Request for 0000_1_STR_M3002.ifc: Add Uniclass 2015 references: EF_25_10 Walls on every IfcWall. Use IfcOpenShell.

First a look at what the model holds.

```python
import ifcopenshell

model = ifcopenshell.open("0000_1_STR_M3002.ifc")
print(model.schema)
print("classifications:", [c.Name for c in model.by_type("IfcClassification")])
for ifc_class in ("IfcDoor", "IfcRoof", "IfcStair", "IfcWall", "IfcWindow"):
    print(ifc_class, len(model.by_type(ifc_class)))
```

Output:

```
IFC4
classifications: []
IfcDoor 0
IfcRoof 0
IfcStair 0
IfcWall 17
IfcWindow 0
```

```python
import ifcopenshell
import ifcopenshell.api.classification

model = ifcopenshell.open("0000_1_STR_M3002.ifc")

system = ifcopenshell.api.classification.add_classification(model, classification="Uniclass 2015")

codes = {
    "IfcWall": ("EF_25_10", "Walls"),
}
for ifc_class, (code, name) in codes.items():
    products = model.by_type(ifc_class)
    ifcopenshell.api.classification.add_reference(
        model, products=products, classification=system, identification=code, name=name
    )
    print(code, len(products))

model.write("0000_1_STR_M3002_edited.ifc")
```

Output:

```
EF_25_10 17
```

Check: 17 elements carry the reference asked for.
